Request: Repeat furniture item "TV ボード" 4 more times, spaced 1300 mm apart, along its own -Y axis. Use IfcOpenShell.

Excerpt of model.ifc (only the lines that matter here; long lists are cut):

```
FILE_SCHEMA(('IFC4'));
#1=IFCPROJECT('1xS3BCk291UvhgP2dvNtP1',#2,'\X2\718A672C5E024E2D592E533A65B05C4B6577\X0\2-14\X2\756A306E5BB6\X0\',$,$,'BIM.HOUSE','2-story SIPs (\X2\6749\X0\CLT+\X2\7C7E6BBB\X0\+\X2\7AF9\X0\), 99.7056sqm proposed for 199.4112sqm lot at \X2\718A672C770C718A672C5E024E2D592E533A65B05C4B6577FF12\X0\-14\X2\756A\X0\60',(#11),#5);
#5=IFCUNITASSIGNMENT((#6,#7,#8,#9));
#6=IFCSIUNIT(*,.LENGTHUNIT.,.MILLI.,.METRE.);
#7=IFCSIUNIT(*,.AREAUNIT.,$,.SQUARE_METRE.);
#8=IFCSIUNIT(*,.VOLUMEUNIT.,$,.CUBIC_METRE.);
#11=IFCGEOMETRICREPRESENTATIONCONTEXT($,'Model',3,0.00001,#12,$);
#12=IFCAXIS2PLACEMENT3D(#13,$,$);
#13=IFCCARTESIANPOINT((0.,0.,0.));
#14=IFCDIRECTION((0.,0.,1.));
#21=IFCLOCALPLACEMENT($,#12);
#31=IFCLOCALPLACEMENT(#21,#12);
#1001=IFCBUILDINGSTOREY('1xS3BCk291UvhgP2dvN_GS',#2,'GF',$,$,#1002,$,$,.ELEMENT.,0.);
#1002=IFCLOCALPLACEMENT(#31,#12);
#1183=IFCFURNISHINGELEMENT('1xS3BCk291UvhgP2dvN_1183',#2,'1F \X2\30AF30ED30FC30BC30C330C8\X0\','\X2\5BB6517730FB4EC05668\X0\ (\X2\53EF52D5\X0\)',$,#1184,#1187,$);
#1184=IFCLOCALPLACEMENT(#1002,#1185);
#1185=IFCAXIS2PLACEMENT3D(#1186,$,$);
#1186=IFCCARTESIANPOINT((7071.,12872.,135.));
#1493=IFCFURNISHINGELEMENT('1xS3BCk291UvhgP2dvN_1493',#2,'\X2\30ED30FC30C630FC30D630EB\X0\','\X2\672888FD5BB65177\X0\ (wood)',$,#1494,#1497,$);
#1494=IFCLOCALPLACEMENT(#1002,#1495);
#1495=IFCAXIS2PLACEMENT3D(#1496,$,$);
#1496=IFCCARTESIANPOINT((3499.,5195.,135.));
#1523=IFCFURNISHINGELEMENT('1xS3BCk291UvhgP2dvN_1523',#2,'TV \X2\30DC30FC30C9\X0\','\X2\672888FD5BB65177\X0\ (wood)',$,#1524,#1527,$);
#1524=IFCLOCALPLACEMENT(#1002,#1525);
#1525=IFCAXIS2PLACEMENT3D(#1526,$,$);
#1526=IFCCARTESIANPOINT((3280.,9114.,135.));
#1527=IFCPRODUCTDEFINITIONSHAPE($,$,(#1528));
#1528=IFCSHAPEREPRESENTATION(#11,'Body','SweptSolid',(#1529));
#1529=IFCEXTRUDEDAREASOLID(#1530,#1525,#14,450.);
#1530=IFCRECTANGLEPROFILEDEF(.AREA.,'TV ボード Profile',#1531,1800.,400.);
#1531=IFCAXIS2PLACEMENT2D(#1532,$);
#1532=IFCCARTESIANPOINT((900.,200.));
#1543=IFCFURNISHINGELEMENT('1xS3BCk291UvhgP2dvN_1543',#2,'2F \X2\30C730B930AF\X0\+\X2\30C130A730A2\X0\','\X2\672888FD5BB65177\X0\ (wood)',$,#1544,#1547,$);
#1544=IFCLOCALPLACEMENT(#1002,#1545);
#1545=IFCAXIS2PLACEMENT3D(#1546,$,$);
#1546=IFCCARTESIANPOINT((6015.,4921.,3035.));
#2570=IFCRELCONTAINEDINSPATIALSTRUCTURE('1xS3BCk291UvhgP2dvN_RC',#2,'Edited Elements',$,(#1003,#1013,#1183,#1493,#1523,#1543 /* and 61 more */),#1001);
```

```python
import ifcopenshell
import ifcopenshell.api.geometry
import ifcopenshell.api.root
import ifcopenshell.util.element
import ifcopenshell.util.placement
import ifcopenshell.util.unit

model = ifcopenshell.open("model.ifc")
unit_scale = ifcopenshell.util.unit.calculate_unit_scale(model)


def reuse_history(source, copy):
    """copy_class also copies each property set's owner history, people and application; keep the originals."""
    for rel in copy.IsDefinedBy:
        if rel.is_a("IfcRelDefinesByProperties") and (history := rel.RelatingPropertyDefinition.OwnerHistory):
            rel.RelatingPropertyDefinition.OwnerHistory = source.OwnerHistory
            ifcopenshell.util.element.remove_deep2(model, history)


source = model.by_guid("1xS3BCk291UvhgP2dvN_1523")
base = ifcopenshell.util.placement.get_local_placement(source.ObjectPlacement)
step = -base[:3, 1] * 1.3 / unit_scale

for i in range(1, 5):
    copy = ifcopenshell.api.root.copy_class(model, product=source)
    copy.Representation = ifcopenshell.util.element.copy_deep(
        model, source.Representation, exclude=["IfcGeometricRepresentationContext", "IfcRepresentationMap"]
    )
    reuse_history(source, copy)
    matrix = base.copy()
    matrix[:3, 3] += i * step
    print("added at", matrix[:3, 3].round(3) + 0.0)
    ifcopenshell.api.geometry.edit_object_placement(model, product=copy, matrix=matrix, is_si=False)

model.write("model_v2.ifc")
```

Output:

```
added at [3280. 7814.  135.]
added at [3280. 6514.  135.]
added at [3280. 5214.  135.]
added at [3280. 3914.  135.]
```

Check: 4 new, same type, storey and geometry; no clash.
